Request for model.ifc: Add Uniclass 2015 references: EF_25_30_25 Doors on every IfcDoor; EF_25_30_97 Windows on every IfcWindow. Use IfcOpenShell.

First a look at what the model holds.

```python
import ifcopenshell

model = ifcopenshell.open("model.ifc")
print(model.schema)
print("classifications:", [c.Name for c in model.by_type("IfcClassification")])
for ifc_class in ("IfcDoor", "IfcRoof", "IfcStair", "IfcWall", "IfcWindow"):
    print(ifc_class, len(model.by_type(ifc_class)))
```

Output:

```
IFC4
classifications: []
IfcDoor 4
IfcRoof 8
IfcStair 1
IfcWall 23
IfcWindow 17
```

```python
import ifcopenshell
import ifcopenshell.api.classification

model = ifcopenshell.open("model.ifc")

system = ifcopenshell.api.classification.add_classification(model, classification="Uniclass 2015")

codes = {
    "IfcDoor": ("EF_25_30_25", "Doors"),
    "IfcWindow": ("EF_25_30_97", "Windows"),
}
for ifc_class, (code, name) in codes.items():
    products = model.by_type(ifc_class)
    ifcopenshell.api.classification.add_reference(
        model, products=products, classification=system, identification=code, name=name
    )
    print(code, len(products))

model.write("model_v2.ifc")
```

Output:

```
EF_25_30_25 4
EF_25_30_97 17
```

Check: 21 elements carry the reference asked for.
